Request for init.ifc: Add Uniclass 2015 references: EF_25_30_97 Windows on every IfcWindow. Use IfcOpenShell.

First a look at what the model holds.

```python
import ifcopenshell

model = ifcopenshell.open("init.ifc")
print(model.schema)
print("classifications:", [c.Name for c in model.by_type("IfcClassification")])
for ifc_class in ("IfcDoor", "IfcRoof", "IfcStair", "IfcWall", "IfcWindow"):
    print(ifc_class, len(model.by_type(ifc_class)))
```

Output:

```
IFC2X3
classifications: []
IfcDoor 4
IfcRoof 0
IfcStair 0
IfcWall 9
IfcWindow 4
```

```python
import ifcopenshell
import ifcopenshell.api.classification

model = ifcopenshell.open("init.ifc")

# IFC2X3 requires Source and Edition and has no link from the project to the system.
system = model.create_entity("IfcClassification", Source="NBS", Edition="2015", Name="Uniclass 2015")

codes = {
    "IfcWindow": ("EF_25_30_97", "Windows"),
}
for ifc_class, (code, name) in codes.items():
    products = model.by_type(ifc_class)
    ifcopenshell.api.classification.add_reference(
        model, products=products, classification=system, identification=code, name=name
    )
    print(code, len(products))

model.write("init_v2.ifc")
```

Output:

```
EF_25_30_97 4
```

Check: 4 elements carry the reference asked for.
